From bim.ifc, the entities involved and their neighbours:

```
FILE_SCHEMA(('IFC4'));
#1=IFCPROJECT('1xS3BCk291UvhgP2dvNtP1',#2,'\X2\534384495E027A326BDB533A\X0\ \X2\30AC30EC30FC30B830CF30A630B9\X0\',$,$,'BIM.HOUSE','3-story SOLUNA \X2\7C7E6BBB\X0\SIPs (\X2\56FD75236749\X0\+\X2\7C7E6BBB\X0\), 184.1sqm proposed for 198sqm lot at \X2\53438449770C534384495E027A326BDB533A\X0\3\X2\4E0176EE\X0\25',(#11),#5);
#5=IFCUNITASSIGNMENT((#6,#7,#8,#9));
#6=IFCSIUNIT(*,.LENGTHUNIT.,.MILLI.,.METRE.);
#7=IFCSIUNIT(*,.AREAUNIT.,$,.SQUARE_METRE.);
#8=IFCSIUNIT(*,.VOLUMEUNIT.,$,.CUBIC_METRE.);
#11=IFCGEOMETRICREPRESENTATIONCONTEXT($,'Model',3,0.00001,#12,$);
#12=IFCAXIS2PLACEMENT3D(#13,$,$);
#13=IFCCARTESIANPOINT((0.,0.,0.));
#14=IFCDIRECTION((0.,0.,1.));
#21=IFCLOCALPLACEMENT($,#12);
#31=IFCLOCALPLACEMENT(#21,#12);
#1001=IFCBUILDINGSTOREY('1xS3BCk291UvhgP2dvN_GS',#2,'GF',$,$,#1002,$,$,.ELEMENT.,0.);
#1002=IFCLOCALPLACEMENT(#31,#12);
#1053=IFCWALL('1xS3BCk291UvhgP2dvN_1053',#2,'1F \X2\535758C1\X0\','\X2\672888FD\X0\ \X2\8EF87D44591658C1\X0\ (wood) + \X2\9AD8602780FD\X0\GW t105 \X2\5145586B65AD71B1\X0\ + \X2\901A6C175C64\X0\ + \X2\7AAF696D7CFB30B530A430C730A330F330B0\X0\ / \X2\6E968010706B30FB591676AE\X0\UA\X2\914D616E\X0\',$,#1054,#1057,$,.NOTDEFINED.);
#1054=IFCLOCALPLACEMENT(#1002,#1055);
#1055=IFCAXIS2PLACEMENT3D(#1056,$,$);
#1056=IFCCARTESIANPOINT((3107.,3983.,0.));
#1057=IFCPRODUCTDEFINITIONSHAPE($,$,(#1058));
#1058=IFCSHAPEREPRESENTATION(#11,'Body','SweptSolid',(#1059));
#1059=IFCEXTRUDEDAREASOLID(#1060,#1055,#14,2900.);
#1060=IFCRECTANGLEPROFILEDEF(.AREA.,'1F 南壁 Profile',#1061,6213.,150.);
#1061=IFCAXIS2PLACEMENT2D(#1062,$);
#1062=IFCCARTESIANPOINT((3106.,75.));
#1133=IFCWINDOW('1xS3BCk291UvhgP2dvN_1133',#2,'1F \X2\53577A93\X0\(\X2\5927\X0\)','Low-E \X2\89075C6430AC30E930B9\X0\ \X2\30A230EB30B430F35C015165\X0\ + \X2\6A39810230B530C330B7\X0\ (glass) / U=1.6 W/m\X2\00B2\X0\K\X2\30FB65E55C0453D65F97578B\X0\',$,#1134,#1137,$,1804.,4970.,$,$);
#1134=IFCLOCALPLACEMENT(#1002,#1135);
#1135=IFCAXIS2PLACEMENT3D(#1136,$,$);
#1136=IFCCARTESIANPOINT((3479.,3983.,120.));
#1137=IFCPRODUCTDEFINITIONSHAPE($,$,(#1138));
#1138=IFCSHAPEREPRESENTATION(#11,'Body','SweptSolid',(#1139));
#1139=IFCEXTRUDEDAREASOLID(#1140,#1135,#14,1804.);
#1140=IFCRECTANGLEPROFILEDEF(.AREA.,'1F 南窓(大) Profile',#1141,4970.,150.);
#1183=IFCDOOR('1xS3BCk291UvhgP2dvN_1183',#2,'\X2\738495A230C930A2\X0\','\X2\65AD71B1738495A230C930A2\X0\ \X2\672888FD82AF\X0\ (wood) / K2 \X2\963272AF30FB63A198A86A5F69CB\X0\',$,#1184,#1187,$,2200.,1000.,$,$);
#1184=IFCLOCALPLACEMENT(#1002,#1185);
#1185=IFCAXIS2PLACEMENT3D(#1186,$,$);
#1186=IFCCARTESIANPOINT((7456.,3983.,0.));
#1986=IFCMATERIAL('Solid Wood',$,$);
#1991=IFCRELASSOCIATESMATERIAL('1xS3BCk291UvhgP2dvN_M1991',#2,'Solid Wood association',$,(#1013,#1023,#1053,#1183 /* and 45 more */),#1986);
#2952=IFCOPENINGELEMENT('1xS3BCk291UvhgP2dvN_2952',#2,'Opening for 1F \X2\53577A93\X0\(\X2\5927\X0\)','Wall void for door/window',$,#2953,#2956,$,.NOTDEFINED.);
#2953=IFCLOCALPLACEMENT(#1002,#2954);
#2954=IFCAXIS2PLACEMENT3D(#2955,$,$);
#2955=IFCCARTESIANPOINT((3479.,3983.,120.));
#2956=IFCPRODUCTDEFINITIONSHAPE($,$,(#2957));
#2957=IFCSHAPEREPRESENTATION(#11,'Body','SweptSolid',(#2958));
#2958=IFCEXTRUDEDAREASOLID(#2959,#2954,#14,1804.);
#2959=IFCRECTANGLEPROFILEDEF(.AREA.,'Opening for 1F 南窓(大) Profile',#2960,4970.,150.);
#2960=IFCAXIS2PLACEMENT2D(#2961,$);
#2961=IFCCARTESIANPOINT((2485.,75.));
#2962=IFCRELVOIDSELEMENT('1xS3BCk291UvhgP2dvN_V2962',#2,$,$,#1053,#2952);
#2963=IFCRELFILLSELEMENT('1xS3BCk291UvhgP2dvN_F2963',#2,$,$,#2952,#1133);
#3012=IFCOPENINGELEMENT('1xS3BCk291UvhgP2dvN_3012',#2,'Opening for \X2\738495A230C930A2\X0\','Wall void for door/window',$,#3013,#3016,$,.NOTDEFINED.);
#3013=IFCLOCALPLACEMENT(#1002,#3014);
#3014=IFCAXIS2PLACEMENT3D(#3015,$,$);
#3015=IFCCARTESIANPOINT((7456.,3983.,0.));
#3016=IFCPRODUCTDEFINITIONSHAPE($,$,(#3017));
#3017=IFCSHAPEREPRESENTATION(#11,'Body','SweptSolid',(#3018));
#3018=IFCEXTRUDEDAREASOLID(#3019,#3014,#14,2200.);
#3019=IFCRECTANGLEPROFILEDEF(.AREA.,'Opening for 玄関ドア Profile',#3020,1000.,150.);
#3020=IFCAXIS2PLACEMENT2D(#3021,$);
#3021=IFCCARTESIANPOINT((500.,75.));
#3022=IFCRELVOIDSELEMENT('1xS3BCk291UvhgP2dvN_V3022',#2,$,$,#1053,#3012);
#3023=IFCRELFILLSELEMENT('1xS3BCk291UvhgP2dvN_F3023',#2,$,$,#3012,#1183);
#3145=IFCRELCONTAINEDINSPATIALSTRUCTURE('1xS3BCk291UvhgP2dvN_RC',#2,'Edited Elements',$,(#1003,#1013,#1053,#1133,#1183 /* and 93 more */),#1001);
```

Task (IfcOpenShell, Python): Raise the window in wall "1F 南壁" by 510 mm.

```python
import numpy as np
import ifcopenshell
import ifcopenshell.api.geometry
import ifcopenshell.util.placement
import ifcopenshell.util.unit

model = ifcopenshell.open("bim.ifc")
unit_scale = ifcopenshell.util.unit.calculate_unit_scale(model)

window = model.by_guid("1xS3BCk291UvhgP2dvN_1133")
opening = window.FillsVoids[0].RelatingOpeningElement
dz = 0.51 / unit_scale

shift = np.array([0.0, 0.0, dz])
# The window is not placed relative to its opening, so move both.
for product in (opening, window):
    matrix = ifcopenshell.util.placement.get_local_placement(product.ObjectPlacement)
    matrix[:3, 3] += shift
    ifcopenshell.api.geometry.edit_object_placement(model, product=product, matrix=matrix, is_si=False)

print(f"moved by {dz * unit_scale:+.3f} m")

model.write("bim_v2.ifc")
```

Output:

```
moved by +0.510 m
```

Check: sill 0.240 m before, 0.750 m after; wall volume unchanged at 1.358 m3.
